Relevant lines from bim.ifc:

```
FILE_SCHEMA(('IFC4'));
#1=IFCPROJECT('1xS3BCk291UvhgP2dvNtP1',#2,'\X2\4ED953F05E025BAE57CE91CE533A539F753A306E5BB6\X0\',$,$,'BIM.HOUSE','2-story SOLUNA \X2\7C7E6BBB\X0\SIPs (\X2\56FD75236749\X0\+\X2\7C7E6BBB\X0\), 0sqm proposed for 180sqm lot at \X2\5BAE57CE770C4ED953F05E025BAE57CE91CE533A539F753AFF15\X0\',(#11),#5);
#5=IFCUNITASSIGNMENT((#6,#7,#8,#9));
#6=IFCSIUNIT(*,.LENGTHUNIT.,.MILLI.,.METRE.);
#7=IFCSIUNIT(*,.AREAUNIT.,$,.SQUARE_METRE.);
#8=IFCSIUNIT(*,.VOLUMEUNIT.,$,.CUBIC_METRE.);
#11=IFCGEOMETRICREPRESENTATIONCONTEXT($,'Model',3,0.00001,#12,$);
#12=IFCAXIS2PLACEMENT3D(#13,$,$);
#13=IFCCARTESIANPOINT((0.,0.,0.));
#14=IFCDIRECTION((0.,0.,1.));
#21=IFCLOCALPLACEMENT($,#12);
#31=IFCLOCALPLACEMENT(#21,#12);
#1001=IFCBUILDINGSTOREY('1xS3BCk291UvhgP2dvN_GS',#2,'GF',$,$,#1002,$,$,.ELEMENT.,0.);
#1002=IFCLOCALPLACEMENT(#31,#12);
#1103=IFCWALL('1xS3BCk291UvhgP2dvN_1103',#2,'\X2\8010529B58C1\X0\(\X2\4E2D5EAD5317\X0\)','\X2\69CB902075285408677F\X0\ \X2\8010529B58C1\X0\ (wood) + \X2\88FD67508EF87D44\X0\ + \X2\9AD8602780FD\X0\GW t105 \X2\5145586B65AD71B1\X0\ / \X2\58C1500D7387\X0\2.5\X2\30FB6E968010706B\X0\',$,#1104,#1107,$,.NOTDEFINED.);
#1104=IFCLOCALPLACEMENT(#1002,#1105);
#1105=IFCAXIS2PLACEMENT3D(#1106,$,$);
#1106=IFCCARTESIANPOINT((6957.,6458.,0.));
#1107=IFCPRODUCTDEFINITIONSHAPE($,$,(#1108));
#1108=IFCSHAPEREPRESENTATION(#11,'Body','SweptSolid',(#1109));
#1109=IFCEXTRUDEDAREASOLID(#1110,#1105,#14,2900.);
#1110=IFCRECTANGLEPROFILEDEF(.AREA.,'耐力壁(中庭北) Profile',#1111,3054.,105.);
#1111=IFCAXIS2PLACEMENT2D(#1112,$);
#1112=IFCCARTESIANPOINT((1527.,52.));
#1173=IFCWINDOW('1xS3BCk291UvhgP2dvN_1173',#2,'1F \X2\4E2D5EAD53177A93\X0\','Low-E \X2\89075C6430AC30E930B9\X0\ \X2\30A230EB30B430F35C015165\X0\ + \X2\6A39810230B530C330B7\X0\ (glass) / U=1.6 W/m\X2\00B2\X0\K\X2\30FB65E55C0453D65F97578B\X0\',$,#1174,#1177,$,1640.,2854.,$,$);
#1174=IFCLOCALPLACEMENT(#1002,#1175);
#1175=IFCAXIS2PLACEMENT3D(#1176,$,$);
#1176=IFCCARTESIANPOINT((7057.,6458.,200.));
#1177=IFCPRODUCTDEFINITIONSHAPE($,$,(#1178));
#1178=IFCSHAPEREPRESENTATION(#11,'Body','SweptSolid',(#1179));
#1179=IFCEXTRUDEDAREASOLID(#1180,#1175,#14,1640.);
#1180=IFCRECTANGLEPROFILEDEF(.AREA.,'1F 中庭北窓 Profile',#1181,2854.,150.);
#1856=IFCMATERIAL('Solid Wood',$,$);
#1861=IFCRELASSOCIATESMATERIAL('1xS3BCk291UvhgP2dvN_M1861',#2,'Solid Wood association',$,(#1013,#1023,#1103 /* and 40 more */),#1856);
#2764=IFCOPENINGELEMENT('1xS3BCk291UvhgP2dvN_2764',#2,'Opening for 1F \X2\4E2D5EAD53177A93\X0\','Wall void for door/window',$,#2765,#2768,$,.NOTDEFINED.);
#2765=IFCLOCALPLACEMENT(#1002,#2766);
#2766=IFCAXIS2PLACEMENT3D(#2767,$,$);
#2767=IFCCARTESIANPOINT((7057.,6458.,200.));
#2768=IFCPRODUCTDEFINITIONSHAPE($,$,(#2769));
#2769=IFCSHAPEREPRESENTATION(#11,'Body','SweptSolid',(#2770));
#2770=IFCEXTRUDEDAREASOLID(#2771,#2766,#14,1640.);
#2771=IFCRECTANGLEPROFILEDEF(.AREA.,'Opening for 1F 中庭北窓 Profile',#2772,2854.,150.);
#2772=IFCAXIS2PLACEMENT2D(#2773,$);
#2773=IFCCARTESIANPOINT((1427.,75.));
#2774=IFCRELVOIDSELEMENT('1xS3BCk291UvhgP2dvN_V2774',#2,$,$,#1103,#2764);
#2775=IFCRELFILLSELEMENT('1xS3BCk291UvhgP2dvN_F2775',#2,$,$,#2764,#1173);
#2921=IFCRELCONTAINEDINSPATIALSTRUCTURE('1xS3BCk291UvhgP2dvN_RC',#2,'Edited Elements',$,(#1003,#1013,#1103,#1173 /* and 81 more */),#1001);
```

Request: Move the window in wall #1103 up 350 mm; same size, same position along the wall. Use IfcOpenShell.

```python
import numpy as np
import ifcopenshell
import ifcopenshell.api.geometry
import ifcopenshell.util.placement
import ifcopenshell.util.unit

model = ifcopenshell.open("bim.ifc")
unit_scale = ifcopenshell.util.unit.calculate_unit_scale(model)

window = model.by_guid("1xS3BCk291UvhgP2dvN_1173")
opening = window.FillsVoids[0].RelatingOpeningElement
dz = 350.0

shift = np.array([0.0, 0.0, dz])
# The window is not placed relative to its opening, so move both.
for product in (opening, window):
    matrix = ifcopenshell.util.placement.get_local_placement(product.ObjectPlacement)
    matrix[:3, 3] += shift
    ifcopenshell.api.geometry.edit_object_placement(model, product=product, matrix=matrix, is_si=False)

print(f"moved by {dz * unit_scale:+.3f} m")

model.write("bim-out.ifc")
```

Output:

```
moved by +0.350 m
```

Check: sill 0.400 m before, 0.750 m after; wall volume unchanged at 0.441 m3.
